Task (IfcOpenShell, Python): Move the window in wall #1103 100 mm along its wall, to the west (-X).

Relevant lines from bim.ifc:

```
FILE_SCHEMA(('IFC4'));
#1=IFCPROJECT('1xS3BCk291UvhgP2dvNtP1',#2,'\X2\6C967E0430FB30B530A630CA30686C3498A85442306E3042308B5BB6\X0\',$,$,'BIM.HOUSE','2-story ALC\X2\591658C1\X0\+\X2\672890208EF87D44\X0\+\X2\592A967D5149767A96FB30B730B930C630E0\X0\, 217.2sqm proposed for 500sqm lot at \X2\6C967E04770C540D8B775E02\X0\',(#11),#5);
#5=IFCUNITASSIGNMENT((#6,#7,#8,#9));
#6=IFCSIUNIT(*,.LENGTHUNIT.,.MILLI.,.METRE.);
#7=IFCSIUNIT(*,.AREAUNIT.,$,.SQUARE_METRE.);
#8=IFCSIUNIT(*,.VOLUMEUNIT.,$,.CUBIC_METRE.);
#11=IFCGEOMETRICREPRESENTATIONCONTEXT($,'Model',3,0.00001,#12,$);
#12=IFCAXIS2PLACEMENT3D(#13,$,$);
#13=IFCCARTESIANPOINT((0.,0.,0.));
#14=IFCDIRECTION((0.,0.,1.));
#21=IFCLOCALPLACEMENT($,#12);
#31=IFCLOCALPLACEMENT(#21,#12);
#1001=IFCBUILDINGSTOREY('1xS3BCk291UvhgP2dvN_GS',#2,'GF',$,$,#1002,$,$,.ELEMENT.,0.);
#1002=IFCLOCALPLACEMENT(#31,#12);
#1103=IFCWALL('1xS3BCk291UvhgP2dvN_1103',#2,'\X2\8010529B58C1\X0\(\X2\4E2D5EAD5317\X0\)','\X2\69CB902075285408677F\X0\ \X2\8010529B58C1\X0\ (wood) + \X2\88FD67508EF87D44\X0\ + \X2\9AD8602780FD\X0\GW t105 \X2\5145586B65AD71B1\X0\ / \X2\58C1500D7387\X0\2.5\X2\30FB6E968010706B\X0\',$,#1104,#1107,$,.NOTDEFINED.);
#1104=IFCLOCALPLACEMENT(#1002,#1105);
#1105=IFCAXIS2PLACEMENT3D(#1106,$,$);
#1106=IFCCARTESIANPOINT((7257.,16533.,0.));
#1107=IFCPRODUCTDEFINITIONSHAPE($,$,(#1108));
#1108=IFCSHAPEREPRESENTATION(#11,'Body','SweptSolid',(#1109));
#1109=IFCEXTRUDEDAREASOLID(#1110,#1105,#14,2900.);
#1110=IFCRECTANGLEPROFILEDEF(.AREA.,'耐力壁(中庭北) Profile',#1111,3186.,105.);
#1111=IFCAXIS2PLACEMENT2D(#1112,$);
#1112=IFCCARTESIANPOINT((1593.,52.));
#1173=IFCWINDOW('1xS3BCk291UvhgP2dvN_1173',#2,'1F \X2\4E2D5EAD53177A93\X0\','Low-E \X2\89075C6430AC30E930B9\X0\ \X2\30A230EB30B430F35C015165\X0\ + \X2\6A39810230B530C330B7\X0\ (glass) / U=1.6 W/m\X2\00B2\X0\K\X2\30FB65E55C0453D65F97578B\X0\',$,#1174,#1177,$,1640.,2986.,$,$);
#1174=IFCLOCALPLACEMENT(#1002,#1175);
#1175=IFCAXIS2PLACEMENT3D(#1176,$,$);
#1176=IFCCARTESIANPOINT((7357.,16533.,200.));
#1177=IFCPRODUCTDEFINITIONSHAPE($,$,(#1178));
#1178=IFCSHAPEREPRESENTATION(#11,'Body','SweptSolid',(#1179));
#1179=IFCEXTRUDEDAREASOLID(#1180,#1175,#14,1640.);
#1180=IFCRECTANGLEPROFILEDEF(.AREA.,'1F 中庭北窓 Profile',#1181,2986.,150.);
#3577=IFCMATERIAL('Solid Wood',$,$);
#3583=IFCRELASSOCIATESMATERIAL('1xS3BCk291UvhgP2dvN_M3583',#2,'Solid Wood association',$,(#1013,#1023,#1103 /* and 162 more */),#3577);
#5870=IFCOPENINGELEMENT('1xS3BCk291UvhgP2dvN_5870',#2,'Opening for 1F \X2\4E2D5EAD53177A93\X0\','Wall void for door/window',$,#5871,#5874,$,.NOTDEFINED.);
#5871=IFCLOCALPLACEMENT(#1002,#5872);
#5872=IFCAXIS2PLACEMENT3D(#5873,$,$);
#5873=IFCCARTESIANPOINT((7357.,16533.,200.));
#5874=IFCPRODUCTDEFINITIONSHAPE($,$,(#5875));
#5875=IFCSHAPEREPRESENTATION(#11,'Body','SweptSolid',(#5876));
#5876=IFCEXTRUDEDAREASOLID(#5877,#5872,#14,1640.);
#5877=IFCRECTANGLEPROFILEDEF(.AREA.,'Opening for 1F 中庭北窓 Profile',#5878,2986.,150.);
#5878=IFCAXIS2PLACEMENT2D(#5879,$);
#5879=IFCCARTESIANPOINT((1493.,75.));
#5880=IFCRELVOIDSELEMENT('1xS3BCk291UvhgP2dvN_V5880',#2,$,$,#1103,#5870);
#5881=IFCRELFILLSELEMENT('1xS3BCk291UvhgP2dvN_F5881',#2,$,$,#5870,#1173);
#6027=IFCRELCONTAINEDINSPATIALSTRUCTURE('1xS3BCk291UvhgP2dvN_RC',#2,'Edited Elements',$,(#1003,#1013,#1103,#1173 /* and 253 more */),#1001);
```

```python
import ifcopenshell
import ifcopenshell.api.geometry
import ifcopenshell.util.placement
import ifcopenshell.util.unit

model = ifcopenshell.open("bim.ifc")
unit_scale = ifcopenshell.util.unit.calculate_unit_scale(model)

window = model.by_guid("1xS3BCk291UvhgP2dvN_1173")
opening = window.FillsVoids[0].RelatingOpeningElement
wall = opening.VoidsElements[0].RelatingBuildingElement

wall_matrix = ifcopenshell.util.placement.get_local_placement(wall.ObjectPlacement)
shift = wall_matrix[:3, 0] * -0.1 / unit_scale
before = ifcopenshell.util.placement.get_local_placement(window.ObjectPlacement)[:3, 3].copy()

# The window is not placed relative to its opening, so move both.
for product in (opening, window):
    matrix = ifcopenshell.util.placement.get_local_placement(product.ObjectPlacement)
    matrix[:3, 3] += shift
    ifcopenshell.api.geometry.edit_object_placement(model, product=product, matrix=matrix, is_si=False)

after = ifcopenshell.util.placement.get_local_placement(window.ObjectPlacement)[:3, 3]
print("window moved by", (after - before).round(3) + 0.0)

model.write("bim_rev.ifc")
```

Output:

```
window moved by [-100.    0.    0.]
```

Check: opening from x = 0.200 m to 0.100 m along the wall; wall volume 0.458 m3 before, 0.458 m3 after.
